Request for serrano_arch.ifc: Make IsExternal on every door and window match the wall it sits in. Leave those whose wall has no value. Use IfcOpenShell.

First a look at what the model holds.

```python
import ifcopenshell
import ifcopenshell.util.element

model = ifcopenshell.open("serrano_arch.ifc")
print(model.schema)
seen = {}
for e in model.by_type("IfcDoor") + model.by_type("IfcWindow"):
    if not e.FillsVoids:
        continue
    host = e.FillsVoids[0].RelatingOpeningElement.VoidsElements[0].RelatingBuildingElement
    own = ifcopenshell.util.element.get_pset(e, f"Pset_{e.is_a()[3:].removesuffix('StandardCase')}Common", "IsExternal")
    wall = ifcopenshell.util.element.get_pset(host, "Pset_WallCommon", "IsExternal")
    seen[e.is_a(), own, wall] = seen.get((e.is_a(), own, wall), 0) + 1
for (cls, own, wall), count in sorted(seen.items(), key=str):
    print(count, cls, "IsExternal:", own, "| host wall:", wall)
```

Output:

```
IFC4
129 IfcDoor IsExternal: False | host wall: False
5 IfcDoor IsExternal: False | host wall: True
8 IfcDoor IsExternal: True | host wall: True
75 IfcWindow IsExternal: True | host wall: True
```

```python
import ifcopenshell
import ifcopenshell.api.pset
import ifcopenshell.util.element

model = ifcopenshell.open("serrano_arch.ifc")

count = 0
for ifc_class, pset_name in (("IfcDoor", "Pset_DoorCommon"), ("IfcWindow", "Pset_WindowCommon")):
    for e in model.by_type(ifc_class):
        if not e.FillsVoids:
            continue
        host = e.FillsVoids[0].RelatingOpeningElement.VoidsElements[0].RelatingBuildingElement
        external = ifcopenshell.util.element.get_pset(host, "Pset_WallCommon", "IsExternal")
        if external is None or ifcopenshell.util.element.get_pset(e, pset_name, "IsExternal") == external:
            continue
        pset = ifcopenshell.api.pset.add_pset(model, product=e, name=pset_name)
        ifcopenshell.api.pset.edit_pset(model, pset=pset, properties={"IsExternal": external})
        count += 1

print(count, "updated")

model.write("serrano_arch-out.ifc")
```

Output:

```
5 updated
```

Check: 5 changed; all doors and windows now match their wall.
